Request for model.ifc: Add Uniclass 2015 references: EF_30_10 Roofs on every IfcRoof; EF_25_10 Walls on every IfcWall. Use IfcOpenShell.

First a look at what the model holds.

```python
import ifcopenshell

model = ifcopenshell.open("model.ifc")
print(model.schema)
print("classifications:", [c.Name for c in model.by_type("IfcClassification")])
for ifc_class in ("IfcDoor", "IfcRoof", "IfcStair", "IfcWall", "IfcWindow"):
    print(ifc_class, len(model.by_type(ifc_class)))
```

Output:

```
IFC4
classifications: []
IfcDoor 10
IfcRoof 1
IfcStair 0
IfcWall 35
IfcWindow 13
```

```python
import ifcopenshell
import ifcopenshell.api.classification

model = ifcopenshell.open("model.ifc")

system = ifcopenshell.api.classification.add_classification(model, classification="Uniclass 2015")

codes = {
    "IfcRoof": ("EF_30_10", "Roofs"),
    "IfcWall": ("EF_25_10", "Walls"),
}
for ifc_class, (code, name) in codes.items():
    products = model.by_type(ifc_class)
    ifcopenshell.api.classification.add_reference(
        model, products=products, classification=system, identification=code, name=name
    )
    print(code, len(products))

model.write("model_rev.ifc")
```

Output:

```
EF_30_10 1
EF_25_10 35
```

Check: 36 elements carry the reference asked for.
